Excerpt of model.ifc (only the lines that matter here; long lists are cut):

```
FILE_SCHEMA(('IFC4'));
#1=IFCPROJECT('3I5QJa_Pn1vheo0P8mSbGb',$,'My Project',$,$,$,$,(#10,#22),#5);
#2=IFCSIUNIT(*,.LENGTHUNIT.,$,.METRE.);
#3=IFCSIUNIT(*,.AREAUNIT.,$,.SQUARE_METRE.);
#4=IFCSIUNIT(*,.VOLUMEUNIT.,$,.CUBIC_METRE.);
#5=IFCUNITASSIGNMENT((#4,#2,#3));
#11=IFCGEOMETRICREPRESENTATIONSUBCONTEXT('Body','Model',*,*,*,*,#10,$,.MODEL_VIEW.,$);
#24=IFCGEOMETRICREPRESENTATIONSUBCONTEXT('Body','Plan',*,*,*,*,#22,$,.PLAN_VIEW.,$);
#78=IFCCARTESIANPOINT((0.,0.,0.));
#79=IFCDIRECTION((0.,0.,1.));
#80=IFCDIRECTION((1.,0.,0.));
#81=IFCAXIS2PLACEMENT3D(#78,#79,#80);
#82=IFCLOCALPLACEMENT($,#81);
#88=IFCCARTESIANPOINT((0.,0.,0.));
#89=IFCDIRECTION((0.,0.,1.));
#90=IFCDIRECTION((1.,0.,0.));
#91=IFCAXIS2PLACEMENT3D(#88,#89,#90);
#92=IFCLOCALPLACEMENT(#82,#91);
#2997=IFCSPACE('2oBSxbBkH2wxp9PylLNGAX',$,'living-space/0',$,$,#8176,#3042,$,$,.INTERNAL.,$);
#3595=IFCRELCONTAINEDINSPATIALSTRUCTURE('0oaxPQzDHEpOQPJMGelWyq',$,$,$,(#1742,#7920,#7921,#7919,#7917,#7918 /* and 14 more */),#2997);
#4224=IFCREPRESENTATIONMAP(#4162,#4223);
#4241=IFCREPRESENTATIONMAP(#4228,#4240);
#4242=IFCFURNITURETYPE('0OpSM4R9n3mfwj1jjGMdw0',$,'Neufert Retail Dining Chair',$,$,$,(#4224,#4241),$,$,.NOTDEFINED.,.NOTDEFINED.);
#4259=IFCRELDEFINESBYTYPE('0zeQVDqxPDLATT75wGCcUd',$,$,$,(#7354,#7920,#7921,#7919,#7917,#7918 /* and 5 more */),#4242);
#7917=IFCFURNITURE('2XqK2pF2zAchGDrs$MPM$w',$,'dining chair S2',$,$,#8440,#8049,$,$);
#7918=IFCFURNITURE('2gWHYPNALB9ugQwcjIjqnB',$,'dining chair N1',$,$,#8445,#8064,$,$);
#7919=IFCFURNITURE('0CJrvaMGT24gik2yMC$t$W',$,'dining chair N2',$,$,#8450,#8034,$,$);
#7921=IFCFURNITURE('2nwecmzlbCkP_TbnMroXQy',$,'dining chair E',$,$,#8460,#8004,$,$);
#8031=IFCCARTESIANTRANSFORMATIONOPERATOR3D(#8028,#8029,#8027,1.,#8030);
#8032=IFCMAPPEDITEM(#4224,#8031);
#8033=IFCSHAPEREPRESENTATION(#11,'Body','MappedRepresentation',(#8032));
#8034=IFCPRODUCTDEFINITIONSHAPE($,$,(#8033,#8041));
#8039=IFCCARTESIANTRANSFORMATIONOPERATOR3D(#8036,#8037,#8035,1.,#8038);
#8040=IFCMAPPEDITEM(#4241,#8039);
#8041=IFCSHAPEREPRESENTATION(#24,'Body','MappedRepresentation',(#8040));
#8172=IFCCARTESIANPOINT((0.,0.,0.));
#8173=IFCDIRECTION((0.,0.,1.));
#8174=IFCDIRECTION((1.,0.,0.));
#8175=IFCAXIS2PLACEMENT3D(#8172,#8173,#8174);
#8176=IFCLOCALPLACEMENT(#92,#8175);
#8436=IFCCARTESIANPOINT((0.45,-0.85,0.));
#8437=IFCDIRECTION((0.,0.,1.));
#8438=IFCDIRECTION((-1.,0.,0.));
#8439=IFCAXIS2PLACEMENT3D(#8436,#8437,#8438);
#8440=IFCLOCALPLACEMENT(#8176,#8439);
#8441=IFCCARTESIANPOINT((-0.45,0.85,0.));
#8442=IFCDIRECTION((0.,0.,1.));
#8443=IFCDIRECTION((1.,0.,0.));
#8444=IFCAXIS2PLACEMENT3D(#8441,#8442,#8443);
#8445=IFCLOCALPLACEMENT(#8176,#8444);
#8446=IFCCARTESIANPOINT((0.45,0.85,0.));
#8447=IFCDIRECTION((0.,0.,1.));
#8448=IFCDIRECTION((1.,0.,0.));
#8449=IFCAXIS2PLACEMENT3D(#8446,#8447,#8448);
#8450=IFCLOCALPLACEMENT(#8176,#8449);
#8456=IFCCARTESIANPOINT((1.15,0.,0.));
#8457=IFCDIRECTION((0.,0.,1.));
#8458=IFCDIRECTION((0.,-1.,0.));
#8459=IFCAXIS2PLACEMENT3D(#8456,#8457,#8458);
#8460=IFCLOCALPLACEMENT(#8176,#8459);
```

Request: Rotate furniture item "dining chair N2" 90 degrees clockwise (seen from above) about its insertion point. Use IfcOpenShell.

```python
import ifcopenshell
import ifcopenshell.api.geometry
import ifcopenshell.util.placement

model = ifcopenshell.open("model.ifc")

item = model.by_guid("0CJrvaMGT24gik2yMC$t$W")
matrix = ifcopenshell.util.placement.get_local_placement(item.ObjectPlacement)
matrix = matrix @ ifcopenshell.util.placement.rotation(-90, "Z")
ifcopenshell.api.geometry.edit_object_placement(model, product=item, matrix=matrix, is_si=False)

print(ifcopenshell.util.placement.get_local_placement(item.ObjectPlacement).round(3) + 0.0)

model.write("model_edited.ifc")
```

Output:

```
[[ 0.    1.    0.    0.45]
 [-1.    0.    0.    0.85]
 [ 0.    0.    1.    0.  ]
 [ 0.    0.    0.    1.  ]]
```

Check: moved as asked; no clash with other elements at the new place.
